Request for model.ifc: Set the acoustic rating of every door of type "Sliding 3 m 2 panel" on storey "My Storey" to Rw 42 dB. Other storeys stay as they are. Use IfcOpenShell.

First a look at what the model holds.

```python
import ifcopenshell
import ifcopenshell.util.element

model = ifcopenshell.open("model.ifc")
print(model.schema)
storey = next(s for s in model.by_type("IfcBuildingStorey") if s.Name == "My Storey")
doors = [e for e in ifcopenshell.util.element.get_decomposition(storey) if e.is_a("IfcDoor")]
seen = {}
for e in doors:
    element_type = ifcopenshell.util.element.get_type(e)
    key = (element_type.Name if element_type != e and element_type else None, ifcopenshell.util.element.get_pset(e, "Pset_DoorCommon", "AcousticRating"))
    seen[key] = seen.get(key, 0) + 1
for (name, value), count in sorted(seen.items(), key=str):
    print(count, "x", name, "|", value)
```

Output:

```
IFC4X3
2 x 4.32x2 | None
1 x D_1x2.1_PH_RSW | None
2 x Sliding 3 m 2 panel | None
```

```python
import ifcopenshell
import ifcopenshell.api.pset
import ifcopenshell.util.element

model = ifcopenshell.open("model.ifc")

storey = next(s for s in model.by_type("IfcBuildingStorey") if s.Name == "My Storey")
doors = [e for e in ifcopenshell.util.element.get_decomposition(storey) if e.is_a("IfcDoor")]

count = 0
for e in doors:
    element_type = ifcopenshell.util.element.get_type(e)
    if element_type in (None, e) or element_type.Name != "Sliding 3 m 2 panel":
        continue
    # add_pset returns the element's existing set when there is one.
    pset = ifcopenshell.api.pset.add_pset(model, product=e, name="Pset_DoorCommon")
    ifcopenshell.api.pset.edit_pset(model, pset=pset, properties={"AcousticRating": "Rw 42 dB"})
    count += 1

print(count, "doors updated")

model.write("model_updated.ifc")
```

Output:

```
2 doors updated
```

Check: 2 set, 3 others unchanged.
